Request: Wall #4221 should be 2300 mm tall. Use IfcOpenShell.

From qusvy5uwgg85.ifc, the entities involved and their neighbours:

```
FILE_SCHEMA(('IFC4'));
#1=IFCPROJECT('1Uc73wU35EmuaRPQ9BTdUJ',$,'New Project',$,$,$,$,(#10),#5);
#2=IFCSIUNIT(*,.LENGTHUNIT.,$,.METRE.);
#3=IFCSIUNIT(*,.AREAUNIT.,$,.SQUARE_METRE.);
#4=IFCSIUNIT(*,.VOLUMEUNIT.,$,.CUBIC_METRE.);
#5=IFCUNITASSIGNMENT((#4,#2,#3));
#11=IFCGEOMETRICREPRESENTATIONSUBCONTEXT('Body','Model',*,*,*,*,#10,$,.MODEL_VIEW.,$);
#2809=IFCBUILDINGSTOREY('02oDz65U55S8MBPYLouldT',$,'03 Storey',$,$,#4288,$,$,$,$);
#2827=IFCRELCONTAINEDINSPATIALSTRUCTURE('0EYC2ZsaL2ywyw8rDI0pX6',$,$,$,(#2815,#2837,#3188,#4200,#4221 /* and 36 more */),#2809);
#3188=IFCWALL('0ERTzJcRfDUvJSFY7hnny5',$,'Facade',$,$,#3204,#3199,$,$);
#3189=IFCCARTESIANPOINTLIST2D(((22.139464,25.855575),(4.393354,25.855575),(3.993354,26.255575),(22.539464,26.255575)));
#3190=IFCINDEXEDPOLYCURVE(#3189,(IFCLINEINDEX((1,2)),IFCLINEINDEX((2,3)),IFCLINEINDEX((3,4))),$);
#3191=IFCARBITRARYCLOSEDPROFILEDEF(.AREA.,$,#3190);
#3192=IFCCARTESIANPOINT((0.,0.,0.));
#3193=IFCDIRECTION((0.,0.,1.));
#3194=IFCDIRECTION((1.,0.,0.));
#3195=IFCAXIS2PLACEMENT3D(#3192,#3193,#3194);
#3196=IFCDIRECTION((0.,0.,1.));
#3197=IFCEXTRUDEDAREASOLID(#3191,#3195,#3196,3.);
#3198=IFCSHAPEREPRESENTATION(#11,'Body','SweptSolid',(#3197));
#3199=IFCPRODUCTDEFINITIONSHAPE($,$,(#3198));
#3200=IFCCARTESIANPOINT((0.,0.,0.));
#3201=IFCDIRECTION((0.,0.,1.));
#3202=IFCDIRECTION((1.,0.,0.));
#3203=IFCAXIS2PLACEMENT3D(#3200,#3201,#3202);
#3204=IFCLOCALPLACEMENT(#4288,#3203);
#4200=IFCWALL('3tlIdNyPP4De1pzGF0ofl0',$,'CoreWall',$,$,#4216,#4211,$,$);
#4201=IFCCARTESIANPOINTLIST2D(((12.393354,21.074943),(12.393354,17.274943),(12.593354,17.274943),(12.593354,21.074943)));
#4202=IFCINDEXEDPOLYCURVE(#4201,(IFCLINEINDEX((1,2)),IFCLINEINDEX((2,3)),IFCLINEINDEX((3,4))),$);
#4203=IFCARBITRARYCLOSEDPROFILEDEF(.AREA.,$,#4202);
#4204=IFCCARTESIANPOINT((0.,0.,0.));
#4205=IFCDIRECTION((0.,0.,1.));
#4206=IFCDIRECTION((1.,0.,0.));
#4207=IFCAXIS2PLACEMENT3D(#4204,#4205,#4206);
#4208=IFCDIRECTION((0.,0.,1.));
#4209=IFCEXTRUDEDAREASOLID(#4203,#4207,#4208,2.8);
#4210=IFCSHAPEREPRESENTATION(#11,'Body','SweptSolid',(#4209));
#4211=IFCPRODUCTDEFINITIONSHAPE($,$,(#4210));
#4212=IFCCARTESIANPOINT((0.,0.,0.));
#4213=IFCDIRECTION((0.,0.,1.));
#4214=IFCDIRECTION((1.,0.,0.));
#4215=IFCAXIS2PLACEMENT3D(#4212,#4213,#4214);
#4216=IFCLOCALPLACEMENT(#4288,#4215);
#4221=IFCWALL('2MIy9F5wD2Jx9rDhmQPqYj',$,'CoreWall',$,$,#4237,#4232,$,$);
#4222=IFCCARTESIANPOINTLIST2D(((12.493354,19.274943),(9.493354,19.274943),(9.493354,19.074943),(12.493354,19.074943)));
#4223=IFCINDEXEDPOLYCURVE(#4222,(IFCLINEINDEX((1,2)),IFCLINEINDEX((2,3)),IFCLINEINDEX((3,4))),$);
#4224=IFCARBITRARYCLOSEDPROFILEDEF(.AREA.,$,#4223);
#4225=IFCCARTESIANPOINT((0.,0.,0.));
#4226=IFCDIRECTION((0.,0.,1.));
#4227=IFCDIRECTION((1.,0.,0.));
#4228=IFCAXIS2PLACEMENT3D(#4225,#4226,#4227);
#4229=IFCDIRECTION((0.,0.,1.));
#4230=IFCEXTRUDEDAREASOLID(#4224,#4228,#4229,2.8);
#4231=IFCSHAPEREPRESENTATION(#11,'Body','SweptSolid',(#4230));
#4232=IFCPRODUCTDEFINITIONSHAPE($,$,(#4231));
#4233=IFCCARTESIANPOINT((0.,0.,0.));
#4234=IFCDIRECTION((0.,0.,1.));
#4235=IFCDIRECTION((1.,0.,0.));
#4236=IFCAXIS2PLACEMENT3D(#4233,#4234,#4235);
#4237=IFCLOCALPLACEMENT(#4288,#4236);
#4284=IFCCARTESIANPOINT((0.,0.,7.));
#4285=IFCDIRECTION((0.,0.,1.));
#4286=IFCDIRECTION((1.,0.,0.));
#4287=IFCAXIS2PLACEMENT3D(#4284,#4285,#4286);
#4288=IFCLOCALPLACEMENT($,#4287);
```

```python
import ifcopenshell
import ifcopenshell.geom
import ifcopenshell.util.representation
import ifcopenshell.util.shape
import ifcopenshell.util.unit

model = ifcopenshell.open("qusvy5uwgg85.ifc")
unit_scale = ifcopenshell.util.unit.calculate_unit_scale(model)
settings = ifcopenshell.geom.settings()


def volume(element):
    """Net volume in cubic metres, openings subtracted."""
    shape = ifcopenshell.geom.create_shape(settings, element)
    return ifcopenshell.util.shape.get_volume(shape.geometry)


wall = model.by_guid("2MIy9F5wD2Jx9rDhmQPqYj")
before = volume(wall)

body = ifcopenshell.util.representation.get_representation(wall, "Model", "Body")
solid = body.Items[0]
old_height = solid.Depth
solid.Depth = 2.3 / unit_scale
after = volume(wall)

print(f"height {old_height:g} -> {solid.Depth:g}, volume {before:.3f} -> {after:.3f} m3")

model.write("qusvy5uwgg85_updated.ifc")
```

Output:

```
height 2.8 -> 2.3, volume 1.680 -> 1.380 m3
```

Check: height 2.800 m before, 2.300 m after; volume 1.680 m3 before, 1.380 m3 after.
